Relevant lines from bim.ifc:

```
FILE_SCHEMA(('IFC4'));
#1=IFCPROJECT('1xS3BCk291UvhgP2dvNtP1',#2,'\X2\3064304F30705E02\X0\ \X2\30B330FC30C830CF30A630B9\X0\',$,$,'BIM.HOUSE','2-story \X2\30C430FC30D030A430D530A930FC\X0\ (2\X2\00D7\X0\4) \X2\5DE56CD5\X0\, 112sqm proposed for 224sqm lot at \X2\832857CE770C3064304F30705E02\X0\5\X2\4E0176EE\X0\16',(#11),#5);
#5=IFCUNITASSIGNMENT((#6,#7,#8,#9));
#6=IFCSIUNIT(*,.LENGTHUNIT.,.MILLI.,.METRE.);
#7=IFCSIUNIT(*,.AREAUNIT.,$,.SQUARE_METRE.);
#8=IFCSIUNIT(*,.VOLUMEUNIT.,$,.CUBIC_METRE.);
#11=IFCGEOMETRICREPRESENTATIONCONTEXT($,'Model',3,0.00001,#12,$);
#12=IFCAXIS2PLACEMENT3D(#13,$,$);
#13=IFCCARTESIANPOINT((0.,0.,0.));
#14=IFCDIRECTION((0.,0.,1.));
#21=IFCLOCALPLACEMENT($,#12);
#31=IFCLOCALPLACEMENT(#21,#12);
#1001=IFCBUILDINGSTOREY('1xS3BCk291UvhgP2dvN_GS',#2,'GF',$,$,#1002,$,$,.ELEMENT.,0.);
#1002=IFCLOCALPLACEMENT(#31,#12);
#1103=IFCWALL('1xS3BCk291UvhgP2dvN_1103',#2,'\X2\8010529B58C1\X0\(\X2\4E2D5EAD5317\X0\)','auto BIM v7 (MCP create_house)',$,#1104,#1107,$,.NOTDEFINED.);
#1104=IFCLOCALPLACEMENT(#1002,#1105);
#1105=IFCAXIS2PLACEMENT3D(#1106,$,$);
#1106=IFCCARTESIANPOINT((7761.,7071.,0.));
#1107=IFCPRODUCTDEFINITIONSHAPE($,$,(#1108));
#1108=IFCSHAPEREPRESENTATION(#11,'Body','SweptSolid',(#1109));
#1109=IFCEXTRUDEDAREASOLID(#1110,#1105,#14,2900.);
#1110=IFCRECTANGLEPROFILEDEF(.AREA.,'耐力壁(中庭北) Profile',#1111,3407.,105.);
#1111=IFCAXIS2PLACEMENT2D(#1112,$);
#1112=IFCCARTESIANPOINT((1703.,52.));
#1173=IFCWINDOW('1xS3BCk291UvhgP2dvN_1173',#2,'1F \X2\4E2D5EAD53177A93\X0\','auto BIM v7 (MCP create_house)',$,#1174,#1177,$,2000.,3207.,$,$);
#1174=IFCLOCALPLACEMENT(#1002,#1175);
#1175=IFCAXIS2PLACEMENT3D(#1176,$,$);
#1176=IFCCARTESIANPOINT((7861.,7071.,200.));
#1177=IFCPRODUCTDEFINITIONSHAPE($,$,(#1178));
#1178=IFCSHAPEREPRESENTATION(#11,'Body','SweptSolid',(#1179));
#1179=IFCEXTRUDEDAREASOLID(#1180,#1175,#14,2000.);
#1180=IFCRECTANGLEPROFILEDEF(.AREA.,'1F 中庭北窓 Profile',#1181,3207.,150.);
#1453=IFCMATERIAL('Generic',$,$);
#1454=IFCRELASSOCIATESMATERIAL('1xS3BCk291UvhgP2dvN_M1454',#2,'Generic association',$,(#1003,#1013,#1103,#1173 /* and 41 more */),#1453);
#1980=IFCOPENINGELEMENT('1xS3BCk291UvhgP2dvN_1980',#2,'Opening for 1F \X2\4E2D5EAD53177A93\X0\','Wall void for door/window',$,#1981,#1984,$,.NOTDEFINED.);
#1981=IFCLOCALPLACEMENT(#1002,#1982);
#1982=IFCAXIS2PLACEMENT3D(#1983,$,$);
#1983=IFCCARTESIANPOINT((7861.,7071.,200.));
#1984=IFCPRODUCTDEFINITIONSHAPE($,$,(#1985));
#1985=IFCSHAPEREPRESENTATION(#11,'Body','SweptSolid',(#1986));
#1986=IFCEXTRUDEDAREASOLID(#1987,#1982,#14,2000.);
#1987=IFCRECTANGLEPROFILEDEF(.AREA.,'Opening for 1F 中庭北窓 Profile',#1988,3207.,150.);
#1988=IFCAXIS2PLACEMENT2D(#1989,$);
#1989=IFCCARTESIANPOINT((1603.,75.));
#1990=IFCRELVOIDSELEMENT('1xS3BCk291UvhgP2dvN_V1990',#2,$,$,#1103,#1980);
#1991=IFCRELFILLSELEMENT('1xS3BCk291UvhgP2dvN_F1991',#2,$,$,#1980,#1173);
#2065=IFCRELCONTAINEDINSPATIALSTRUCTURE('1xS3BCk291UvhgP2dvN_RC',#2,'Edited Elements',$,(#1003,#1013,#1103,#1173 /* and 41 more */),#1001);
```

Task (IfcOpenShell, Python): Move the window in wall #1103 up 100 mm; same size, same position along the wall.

```python
import numpy as np
import ifcopenshell
import ifcopenshell.api.geometry
import ifcopenshell.util.placement
import ifcopenshell.util.unit

model = ifcopenshell.open("bim.ifc")
unit_scale = ifcopenshell.util.unit.calculate_unit_scale(model)

window = model.by_guid("1xS3BCk291UvhgP2dvN_1173")
opening = window.FillsVoids[0].RelatingOpeningElement
dz = 0.1 / unit_scale

shift = np.array([0.0, 0.0, dz])
# The window is not placed relative to its opening, so move both.
for product in (opening, window):
    matrix = ifcopenshell.util.placement.get_local_placement(product.ObjectPlacement)
    matrix[:3, 3] += shift
    ifcopenshell.api.geometry.edit_object_placement(model, product=product, matrix=matrix, is_si=False)

print(f"moved by {dz * unit_scale:+.3f} m")

model.write("bim-out.ifc")
```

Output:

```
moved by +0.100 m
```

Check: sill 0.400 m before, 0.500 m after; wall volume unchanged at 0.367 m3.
